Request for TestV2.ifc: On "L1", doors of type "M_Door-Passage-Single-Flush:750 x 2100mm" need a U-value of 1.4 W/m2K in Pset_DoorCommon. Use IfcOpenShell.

First a look at what the model holds.

```python
import ifcopenshell
import ifcopenshell.util.element

model = ifcopenshell.open("TestV2.ifc")
print(model.schema)
storey = next(s for s in model.by_type("IfcBuildingStorey") if s.Name == "L1")
doors = [e for e in ifcopenshell.util.element.get_decomposition(storey) if e.is_a("IfcDoor")]
seen = {}
for e in doors:
    element_type = ifcopenshell.util.element.get_type(e)
    key = (element_type.Name if element_type != e and element_type else None, ifcopenshell.util.element.get_pset(e, "Pset_DoorCommon", "ThermalTransmittance"))
    seen[key] = seen.get(key, 0) + 1
for (name, value), count in sorted(seen.items(), key=str):
    print(count, "x", name, "|", value)
```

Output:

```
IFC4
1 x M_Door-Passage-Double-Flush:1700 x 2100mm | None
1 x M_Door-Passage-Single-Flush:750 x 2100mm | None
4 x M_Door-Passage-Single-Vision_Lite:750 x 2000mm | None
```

```python
import ifcopenshell
import ifcopenshell.api.pset
import ifcopenshell.util.element

model = ifcopenshell.open("TestV2.ifc")

storey = next(s for s in model.by_type("IfcBuildingStorey") if s.Name == "L1")
doors = [e for e in ifcopenshell.util.element.get_decomposition(storey) if e.is_a("IfcDoor")]

count = 0
for e in doors:
    element_type = ifcopenshell.util.element.get_type(e)
    if element_type in (None, e) or element_type.Name != "M_Door-Passage-Single-Flush:750 x 2100mm":
        continue
    # add_pset returns the element's existing set when there is one.
    pset = ifcopenshell.api.pset.add_pset(model, product=e, name="Pset_DoorCommon")
    ifcopenshell.api.pset.edit_pset(model, pset=pset, properties={"ThermalTransmittance": 1.4})
    count += 1

print(count, "doors updated")

model.write("TestV2_updated.ifc")
```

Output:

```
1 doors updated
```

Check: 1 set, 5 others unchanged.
